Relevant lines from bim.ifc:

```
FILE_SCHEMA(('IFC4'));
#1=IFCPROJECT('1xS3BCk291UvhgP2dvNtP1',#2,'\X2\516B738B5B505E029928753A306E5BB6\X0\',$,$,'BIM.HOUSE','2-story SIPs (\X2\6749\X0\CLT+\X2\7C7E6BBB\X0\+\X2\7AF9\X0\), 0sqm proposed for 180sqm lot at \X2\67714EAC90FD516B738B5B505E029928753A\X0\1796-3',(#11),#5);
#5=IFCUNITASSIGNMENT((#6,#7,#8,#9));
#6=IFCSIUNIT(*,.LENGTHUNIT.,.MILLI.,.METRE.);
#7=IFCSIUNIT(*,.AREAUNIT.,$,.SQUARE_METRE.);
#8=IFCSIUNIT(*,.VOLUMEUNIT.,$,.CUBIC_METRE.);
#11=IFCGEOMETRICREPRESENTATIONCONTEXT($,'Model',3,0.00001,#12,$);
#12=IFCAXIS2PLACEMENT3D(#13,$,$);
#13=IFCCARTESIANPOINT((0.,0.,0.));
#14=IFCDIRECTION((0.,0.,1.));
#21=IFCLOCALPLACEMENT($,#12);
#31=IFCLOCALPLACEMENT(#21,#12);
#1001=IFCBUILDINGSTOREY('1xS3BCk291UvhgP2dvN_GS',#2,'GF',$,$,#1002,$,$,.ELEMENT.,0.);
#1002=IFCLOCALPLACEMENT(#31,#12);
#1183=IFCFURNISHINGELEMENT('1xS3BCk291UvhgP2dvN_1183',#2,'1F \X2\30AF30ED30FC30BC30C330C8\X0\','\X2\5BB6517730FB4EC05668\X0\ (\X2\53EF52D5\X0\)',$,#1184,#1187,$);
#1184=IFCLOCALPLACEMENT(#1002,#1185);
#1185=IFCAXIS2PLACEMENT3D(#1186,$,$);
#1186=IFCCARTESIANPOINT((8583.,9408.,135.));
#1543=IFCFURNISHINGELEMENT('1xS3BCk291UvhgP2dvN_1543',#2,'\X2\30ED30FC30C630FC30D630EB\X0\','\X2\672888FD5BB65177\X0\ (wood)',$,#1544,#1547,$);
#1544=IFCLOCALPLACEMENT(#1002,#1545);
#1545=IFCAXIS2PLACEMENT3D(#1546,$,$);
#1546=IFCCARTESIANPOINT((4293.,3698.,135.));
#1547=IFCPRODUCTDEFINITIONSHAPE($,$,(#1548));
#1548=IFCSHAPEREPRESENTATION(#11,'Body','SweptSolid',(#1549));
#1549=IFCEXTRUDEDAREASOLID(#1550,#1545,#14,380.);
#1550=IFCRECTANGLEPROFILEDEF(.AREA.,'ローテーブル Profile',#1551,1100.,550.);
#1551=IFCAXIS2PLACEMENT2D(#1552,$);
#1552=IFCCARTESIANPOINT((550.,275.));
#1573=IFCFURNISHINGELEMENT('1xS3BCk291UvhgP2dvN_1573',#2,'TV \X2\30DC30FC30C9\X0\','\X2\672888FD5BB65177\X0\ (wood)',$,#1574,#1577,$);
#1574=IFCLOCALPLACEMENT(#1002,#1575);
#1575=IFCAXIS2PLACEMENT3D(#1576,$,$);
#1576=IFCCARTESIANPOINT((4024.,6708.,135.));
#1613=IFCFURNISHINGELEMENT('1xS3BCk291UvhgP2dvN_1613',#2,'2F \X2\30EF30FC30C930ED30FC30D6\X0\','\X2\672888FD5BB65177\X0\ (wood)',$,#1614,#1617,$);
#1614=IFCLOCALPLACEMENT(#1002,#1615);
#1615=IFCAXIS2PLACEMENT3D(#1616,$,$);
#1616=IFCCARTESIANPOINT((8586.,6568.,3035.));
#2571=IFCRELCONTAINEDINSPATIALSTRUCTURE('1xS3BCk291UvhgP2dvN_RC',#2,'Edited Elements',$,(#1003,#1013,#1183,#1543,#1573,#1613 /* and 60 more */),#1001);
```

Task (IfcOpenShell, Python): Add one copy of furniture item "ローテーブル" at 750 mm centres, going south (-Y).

```python
import numpy as np
import ifcopenshell
import ifcopenshell.api.geometry
import ifcopenshell.api.root
import ifcopenshell.util.element
import ifcopenshell.util.placement

model = ifcopenshell.open("bim.ifc")


def reuse_history(source, copy):
    """copy_class also copies each property set's owner history, people and application; keep the originals."""
    for rel in copy.IsDefinedBy:
        if rel.is_a("IfcRelDefinesByProperties") and (history := rel.RelatingPropertyDefinition.OwnerHistory):
            rel.RelatingPropertyDefinition.OwnerHistory = source.OwnerHistory
            ifcopenshell.util.element.remove_deep2(model, history)


source = model.by_guid("1xS3BCk291UvhgP2dvN_1543")
base = ifcopenshell.util.placement.get_local_placement(source.ObjectPlacement)
step = np.array([0.0, -1.0, 0.0]) * 750.0

for i in range(1, 2):
    copy = ifcopenshell.api.root.copy_class(model, product=source)
    copy.Representation = ifcopenshell.util.element.copy_deep(
        model, source.Representation, exclude=["IfcGeometricRepresentationContext", "IfcRepresentationMap"]
    )
    reuse_history(source, copy)
    matrix = base.copy()
    matrix[:3, 3] += i * step
    print("added at", matrix[:3, 3].round(3) + 0.0)
    ifcopenshell.api.geometry.edit_object_placement(model, product=copy, matrix=matrix, is_si=False)

model.write("bim_rev.ifc")
```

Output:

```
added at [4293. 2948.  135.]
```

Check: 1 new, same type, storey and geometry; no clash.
